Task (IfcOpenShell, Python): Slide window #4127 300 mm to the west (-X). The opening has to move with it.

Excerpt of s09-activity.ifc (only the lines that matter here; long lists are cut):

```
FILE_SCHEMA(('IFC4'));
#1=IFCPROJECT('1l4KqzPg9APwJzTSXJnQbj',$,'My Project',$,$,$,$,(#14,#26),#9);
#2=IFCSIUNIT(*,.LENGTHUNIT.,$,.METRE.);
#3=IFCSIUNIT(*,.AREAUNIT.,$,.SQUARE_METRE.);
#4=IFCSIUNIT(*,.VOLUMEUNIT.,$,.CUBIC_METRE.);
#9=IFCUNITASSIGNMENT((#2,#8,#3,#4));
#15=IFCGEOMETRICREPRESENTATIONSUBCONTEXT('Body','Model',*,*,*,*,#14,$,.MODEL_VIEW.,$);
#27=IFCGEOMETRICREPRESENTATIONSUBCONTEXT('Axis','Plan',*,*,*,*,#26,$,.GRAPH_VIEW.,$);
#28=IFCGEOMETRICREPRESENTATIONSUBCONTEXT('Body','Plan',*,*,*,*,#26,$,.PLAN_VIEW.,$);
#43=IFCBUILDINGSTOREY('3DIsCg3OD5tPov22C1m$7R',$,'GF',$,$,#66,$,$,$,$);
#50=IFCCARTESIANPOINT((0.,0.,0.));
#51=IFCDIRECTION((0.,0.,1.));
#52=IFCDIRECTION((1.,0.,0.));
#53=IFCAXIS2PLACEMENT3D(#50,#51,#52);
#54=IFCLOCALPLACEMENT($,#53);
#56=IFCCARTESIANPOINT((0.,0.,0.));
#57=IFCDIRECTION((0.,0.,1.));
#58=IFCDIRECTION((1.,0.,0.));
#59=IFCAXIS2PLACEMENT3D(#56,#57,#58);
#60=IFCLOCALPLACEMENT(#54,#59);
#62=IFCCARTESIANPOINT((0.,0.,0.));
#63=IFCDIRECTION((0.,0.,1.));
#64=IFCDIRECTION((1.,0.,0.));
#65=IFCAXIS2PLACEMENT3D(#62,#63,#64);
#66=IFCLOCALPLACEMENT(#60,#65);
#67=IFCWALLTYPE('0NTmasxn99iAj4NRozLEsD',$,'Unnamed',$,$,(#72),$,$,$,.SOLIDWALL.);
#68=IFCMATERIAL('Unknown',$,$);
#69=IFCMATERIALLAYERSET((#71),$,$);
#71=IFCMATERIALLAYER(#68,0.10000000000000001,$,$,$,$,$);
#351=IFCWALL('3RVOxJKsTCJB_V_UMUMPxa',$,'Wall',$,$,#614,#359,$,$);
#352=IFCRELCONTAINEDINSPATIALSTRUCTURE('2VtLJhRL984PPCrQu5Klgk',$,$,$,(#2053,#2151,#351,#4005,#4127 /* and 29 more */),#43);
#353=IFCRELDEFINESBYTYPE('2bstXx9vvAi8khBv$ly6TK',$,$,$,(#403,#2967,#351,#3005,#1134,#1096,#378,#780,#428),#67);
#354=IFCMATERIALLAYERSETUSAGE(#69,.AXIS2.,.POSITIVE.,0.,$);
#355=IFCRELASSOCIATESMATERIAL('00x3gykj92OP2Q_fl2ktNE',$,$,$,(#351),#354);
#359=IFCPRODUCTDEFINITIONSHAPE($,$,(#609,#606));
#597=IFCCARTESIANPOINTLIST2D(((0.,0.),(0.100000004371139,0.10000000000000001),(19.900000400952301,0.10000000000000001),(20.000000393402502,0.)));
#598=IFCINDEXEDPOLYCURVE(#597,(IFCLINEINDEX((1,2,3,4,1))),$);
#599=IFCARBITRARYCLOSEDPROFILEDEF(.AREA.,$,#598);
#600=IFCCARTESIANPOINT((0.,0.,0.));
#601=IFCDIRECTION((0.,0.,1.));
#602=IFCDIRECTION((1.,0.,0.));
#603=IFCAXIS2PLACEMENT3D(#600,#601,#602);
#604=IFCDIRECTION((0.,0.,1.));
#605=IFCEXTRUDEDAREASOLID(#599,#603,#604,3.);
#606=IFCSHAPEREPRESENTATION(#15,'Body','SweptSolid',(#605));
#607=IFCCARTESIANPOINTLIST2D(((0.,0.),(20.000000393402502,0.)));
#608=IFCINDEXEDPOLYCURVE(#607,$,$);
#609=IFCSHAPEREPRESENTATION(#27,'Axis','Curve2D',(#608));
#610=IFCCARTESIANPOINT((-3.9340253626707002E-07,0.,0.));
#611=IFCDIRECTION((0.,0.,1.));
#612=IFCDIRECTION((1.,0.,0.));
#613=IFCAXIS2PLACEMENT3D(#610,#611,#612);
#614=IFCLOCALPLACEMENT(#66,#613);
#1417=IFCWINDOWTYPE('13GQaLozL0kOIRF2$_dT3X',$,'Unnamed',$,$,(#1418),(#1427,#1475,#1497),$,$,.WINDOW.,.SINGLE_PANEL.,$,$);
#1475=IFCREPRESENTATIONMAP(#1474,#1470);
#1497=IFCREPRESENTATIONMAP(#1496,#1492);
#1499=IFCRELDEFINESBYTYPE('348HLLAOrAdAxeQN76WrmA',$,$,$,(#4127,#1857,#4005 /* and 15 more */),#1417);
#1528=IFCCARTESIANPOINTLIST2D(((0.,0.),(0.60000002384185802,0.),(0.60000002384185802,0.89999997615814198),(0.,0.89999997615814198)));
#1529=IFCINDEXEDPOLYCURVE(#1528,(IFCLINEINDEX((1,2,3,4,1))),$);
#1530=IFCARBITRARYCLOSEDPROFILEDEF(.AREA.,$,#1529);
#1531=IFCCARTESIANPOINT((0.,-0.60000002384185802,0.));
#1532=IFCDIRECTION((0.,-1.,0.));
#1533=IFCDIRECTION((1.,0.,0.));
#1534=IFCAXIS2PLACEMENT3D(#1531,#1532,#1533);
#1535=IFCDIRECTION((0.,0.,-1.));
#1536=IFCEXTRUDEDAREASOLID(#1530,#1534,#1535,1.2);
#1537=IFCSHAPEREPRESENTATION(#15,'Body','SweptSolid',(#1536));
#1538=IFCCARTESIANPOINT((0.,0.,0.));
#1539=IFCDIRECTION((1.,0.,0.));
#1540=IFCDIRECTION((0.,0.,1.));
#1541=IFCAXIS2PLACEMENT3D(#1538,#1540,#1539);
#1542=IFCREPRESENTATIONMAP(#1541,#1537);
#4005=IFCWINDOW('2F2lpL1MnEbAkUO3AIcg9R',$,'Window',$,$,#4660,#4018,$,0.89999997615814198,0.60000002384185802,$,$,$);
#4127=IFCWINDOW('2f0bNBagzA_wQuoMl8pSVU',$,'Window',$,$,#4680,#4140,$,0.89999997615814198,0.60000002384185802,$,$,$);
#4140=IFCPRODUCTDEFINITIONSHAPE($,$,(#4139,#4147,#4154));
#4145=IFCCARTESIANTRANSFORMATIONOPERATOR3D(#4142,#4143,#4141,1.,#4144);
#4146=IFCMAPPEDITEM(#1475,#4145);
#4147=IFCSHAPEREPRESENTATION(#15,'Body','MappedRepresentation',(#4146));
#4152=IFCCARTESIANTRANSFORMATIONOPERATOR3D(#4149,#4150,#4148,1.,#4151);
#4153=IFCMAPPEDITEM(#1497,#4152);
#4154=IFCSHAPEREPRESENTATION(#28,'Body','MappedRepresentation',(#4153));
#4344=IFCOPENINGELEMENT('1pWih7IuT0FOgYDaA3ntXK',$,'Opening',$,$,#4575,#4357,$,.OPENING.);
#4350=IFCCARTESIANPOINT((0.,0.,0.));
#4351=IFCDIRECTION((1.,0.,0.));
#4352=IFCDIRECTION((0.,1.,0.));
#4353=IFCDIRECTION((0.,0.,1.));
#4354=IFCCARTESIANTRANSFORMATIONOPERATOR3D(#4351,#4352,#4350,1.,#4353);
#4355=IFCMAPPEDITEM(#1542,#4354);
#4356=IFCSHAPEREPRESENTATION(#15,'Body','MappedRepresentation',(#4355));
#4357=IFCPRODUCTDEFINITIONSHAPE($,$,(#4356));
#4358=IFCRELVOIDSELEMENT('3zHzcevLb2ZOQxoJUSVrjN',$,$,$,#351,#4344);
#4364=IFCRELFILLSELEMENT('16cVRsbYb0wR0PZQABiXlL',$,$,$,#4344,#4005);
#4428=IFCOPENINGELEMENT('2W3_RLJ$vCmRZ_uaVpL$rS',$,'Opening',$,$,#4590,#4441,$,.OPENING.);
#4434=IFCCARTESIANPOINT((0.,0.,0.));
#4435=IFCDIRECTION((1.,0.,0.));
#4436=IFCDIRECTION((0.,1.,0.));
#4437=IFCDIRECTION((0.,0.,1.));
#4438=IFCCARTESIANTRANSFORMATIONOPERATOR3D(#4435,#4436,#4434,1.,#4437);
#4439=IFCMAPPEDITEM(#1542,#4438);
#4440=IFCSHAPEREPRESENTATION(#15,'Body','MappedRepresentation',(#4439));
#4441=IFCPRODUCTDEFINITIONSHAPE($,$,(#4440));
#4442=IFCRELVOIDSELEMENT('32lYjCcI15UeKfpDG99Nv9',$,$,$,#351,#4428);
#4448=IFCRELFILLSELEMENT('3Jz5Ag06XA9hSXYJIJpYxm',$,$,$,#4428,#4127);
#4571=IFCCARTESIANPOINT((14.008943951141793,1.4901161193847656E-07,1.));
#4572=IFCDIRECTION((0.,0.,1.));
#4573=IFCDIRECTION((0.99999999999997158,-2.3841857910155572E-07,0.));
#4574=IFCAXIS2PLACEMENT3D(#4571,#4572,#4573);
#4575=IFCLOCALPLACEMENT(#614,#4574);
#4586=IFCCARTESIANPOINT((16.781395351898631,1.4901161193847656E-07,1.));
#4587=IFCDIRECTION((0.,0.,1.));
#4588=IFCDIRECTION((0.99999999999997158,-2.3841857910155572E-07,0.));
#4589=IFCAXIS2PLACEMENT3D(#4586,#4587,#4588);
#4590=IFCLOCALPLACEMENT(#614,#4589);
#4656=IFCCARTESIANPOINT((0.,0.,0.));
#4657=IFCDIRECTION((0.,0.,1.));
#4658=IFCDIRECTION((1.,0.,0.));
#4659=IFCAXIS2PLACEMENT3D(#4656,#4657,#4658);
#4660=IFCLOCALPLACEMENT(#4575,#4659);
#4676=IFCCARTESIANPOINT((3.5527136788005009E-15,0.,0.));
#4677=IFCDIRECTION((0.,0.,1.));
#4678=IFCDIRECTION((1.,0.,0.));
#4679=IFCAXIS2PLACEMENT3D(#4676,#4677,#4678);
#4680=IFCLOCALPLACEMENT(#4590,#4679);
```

```python
import ifcopenshell
import ifcopenshell.api.geometry
import ifcopenshell.util.placement
import ifcopenshell.util.unit

model = ifcopenshell.open("s09-activity.ifc")
unit_scale = ifcopenshell.util.unit.calculate_unit_scale(model)

window = model.by_id(4127)
opening = window.FillsVoids[0].RelatingOpeningElement
wall = opening.VoidsElements[0].RelatingBuildingElement

wall_matrix = ifcopenshell.util.placement.get_local_placement(wall.ObjectPlacement)
shift = wall_matrix[:3, 0] * -0.3 / unit_scale
before = ifcopenshell.util.placement.get_local_placement(window.ObjectPlacement)[:3, 3].copy()

# The window is placed relative to its opening, so it follows when the opening moves.
matrix = ifcopenshell.util.placement.get_local_placement(opening.ObjectPlacement)
matrix[:3, 3] += shift
ifcopenshell.api.geometry.edit_object_placement(
    model, product=opening, matrix=matrix, is_si=False, should_transform_children=True
)

after = ifcopenshell.util.placement.get_local_placement(window.ObjectPlacement)[:3, 3]
print("window moved by", (after - before).round(3) + 0.0)

model.write("s09-activity_rev.ifc")
```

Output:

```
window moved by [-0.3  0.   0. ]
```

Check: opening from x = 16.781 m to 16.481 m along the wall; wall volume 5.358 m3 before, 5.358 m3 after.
